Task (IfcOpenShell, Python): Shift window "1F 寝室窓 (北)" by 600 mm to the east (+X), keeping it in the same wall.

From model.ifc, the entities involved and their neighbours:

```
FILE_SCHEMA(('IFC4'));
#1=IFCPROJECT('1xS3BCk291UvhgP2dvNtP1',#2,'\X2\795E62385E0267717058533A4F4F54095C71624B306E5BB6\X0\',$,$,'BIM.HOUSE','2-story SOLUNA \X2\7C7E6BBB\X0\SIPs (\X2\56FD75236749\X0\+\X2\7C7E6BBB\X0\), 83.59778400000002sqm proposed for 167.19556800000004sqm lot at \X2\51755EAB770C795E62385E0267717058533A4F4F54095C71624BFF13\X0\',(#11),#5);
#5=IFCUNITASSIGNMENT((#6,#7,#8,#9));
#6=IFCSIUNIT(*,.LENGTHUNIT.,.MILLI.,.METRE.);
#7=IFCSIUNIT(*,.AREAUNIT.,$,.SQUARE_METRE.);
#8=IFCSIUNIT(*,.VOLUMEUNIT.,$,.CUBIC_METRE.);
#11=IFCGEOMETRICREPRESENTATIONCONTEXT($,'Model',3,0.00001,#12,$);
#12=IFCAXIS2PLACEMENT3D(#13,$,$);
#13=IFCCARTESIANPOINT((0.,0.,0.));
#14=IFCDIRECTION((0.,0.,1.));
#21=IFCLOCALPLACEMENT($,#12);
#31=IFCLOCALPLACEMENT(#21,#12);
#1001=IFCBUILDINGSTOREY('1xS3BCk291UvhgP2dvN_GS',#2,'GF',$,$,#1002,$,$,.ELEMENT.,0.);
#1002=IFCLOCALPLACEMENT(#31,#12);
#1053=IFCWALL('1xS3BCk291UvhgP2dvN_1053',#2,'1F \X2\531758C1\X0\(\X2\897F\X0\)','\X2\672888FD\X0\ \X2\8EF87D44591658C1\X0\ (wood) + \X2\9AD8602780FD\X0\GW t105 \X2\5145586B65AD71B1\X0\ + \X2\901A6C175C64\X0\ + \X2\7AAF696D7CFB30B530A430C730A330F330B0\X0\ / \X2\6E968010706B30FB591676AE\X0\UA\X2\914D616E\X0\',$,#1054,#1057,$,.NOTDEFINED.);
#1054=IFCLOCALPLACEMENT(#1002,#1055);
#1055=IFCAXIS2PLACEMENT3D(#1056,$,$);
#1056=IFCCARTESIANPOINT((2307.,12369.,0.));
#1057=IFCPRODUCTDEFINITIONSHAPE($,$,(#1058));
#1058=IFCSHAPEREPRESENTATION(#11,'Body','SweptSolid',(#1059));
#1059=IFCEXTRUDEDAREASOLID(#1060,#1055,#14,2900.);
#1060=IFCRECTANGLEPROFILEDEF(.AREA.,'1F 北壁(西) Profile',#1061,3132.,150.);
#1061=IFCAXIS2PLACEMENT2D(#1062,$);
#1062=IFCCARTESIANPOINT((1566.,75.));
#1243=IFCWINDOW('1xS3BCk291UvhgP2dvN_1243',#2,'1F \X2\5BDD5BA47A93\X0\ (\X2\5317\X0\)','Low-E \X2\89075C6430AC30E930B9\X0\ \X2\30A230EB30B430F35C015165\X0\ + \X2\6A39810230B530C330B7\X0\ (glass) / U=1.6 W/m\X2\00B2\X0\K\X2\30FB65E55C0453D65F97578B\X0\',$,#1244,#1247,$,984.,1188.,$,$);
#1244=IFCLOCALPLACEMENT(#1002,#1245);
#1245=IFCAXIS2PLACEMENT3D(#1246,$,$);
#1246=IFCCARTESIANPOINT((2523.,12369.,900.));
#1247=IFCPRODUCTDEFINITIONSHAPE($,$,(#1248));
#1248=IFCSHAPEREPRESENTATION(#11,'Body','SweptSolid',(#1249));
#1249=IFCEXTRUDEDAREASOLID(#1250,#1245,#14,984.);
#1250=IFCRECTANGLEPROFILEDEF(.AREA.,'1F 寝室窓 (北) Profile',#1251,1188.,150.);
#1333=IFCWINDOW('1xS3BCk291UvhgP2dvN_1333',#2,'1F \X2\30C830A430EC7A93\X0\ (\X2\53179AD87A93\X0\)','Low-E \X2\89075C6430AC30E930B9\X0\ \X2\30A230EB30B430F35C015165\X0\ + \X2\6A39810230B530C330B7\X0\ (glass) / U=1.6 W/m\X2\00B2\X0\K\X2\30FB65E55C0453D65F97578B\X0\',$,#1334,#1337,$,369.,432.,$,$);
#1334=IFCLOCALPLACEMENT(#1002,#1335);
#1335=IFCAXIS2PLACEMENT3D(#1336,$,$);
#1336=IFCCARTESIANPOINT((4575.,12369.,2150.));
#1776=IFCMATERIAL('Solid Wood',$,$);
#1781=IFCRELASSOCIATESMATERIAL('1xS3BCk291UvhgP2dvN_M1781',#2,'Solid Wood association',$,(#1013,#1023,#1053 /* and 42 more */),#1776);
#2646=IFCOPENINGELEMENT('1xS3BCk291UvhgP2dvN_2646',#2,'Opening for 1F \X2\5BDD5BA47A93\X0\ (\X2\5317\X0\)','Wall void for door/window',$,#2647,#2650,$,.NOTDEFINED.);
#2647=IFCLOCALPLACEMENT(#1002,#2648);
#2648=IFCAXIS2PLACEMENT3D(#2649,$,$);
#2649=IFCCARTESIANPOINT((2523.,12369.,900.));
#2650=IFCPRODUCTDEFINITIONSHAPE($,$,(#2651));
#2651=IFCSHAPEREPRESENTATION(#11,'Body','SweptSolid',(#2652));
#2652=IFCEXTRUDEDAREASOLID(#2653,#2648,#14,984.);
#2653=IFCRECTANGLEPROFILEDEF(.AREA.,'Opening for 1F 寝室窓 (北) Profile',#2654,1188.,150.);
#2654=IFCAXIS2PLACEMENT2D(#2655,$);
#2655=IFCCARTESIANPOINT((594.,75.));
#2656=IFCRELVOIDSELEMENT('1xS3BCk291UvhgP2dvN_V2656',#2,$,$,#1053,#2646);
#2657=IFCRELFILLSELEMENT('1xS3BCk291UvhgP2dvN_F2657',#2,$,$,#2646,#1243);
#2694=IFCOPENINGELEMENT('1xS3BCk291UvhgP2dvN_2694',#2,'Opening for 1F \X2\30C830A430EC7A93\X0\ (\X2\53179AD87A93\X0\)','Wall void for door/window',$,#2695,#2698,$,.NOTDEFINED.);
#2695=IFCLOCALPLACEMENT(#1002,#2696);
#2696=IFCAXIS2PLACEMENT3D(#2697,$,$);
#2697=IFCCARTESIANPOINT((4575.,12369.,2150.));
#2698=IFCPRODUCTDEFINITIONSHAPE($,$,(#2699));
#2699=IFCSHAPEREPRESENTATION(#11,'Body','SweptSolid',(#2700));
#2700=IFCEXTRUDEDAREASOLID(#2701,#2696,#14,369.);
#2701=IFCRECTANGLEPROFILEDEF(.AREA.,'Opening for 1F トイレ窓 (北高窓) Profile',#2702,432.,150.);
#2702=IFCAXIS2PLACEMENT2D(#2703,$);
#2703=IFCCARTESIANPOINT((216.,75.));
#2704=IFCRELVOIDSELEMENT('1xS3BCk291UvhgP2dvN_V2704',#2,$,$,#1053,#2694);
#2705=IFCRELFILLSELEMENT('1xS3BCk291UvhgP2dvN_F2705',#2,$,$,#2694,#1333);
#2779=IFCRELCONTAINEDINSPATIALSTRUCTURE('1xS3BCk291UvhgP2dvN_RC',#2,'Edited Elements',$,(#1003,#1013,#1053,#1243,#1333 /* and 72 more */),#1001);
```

```python
import ifcopenshell
import ifcopenshell.api.geometry
import ifcopenshell.util.placement
import ifcopenshell.util.unit

model = ifcopenshell.open("model.ifc")
unit_scale = ifcopenshell.util.unit.calculate_unit_scale(model)

window = model.by_id(1243)
opening = window.FillsVoids[0].RelatingOpeningElement
wall = opening.VoidsElements[0].RelatingBuildingElement

wall_matrix = ifcopenshell.util.placement.get_local_placement(wall.ObjectPlacement)
shift = wall_matrix[:3, 0] * 0.6 / unit_scale
before = ifcopenshell.util.placement.get_local_placement(window.ObjectPlacement)[:3, 3].copy()

# The window is not placed relative to its opening, so move both.
for product in (opening, window):
    matrix = ifcopenshell.util.placement.get_local_placement(product.ObjectPlacement)
    matrix[:3, 3] += shift
    ifcopenshell.api.geometry.edit_object_placement(model, product=product, matrix=matrix, is_si=False)

after = ifcopenshell.util.placement.get_local_placement(window.ObjectPlacement)[:3, 3]
print("window moved by", (after - before).round(3) + 0.0)

model.write("model_edited.ifc")
```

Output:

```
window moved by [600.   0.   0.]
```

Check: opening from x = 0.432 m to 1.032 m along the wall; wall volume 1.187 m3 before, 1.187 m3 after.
